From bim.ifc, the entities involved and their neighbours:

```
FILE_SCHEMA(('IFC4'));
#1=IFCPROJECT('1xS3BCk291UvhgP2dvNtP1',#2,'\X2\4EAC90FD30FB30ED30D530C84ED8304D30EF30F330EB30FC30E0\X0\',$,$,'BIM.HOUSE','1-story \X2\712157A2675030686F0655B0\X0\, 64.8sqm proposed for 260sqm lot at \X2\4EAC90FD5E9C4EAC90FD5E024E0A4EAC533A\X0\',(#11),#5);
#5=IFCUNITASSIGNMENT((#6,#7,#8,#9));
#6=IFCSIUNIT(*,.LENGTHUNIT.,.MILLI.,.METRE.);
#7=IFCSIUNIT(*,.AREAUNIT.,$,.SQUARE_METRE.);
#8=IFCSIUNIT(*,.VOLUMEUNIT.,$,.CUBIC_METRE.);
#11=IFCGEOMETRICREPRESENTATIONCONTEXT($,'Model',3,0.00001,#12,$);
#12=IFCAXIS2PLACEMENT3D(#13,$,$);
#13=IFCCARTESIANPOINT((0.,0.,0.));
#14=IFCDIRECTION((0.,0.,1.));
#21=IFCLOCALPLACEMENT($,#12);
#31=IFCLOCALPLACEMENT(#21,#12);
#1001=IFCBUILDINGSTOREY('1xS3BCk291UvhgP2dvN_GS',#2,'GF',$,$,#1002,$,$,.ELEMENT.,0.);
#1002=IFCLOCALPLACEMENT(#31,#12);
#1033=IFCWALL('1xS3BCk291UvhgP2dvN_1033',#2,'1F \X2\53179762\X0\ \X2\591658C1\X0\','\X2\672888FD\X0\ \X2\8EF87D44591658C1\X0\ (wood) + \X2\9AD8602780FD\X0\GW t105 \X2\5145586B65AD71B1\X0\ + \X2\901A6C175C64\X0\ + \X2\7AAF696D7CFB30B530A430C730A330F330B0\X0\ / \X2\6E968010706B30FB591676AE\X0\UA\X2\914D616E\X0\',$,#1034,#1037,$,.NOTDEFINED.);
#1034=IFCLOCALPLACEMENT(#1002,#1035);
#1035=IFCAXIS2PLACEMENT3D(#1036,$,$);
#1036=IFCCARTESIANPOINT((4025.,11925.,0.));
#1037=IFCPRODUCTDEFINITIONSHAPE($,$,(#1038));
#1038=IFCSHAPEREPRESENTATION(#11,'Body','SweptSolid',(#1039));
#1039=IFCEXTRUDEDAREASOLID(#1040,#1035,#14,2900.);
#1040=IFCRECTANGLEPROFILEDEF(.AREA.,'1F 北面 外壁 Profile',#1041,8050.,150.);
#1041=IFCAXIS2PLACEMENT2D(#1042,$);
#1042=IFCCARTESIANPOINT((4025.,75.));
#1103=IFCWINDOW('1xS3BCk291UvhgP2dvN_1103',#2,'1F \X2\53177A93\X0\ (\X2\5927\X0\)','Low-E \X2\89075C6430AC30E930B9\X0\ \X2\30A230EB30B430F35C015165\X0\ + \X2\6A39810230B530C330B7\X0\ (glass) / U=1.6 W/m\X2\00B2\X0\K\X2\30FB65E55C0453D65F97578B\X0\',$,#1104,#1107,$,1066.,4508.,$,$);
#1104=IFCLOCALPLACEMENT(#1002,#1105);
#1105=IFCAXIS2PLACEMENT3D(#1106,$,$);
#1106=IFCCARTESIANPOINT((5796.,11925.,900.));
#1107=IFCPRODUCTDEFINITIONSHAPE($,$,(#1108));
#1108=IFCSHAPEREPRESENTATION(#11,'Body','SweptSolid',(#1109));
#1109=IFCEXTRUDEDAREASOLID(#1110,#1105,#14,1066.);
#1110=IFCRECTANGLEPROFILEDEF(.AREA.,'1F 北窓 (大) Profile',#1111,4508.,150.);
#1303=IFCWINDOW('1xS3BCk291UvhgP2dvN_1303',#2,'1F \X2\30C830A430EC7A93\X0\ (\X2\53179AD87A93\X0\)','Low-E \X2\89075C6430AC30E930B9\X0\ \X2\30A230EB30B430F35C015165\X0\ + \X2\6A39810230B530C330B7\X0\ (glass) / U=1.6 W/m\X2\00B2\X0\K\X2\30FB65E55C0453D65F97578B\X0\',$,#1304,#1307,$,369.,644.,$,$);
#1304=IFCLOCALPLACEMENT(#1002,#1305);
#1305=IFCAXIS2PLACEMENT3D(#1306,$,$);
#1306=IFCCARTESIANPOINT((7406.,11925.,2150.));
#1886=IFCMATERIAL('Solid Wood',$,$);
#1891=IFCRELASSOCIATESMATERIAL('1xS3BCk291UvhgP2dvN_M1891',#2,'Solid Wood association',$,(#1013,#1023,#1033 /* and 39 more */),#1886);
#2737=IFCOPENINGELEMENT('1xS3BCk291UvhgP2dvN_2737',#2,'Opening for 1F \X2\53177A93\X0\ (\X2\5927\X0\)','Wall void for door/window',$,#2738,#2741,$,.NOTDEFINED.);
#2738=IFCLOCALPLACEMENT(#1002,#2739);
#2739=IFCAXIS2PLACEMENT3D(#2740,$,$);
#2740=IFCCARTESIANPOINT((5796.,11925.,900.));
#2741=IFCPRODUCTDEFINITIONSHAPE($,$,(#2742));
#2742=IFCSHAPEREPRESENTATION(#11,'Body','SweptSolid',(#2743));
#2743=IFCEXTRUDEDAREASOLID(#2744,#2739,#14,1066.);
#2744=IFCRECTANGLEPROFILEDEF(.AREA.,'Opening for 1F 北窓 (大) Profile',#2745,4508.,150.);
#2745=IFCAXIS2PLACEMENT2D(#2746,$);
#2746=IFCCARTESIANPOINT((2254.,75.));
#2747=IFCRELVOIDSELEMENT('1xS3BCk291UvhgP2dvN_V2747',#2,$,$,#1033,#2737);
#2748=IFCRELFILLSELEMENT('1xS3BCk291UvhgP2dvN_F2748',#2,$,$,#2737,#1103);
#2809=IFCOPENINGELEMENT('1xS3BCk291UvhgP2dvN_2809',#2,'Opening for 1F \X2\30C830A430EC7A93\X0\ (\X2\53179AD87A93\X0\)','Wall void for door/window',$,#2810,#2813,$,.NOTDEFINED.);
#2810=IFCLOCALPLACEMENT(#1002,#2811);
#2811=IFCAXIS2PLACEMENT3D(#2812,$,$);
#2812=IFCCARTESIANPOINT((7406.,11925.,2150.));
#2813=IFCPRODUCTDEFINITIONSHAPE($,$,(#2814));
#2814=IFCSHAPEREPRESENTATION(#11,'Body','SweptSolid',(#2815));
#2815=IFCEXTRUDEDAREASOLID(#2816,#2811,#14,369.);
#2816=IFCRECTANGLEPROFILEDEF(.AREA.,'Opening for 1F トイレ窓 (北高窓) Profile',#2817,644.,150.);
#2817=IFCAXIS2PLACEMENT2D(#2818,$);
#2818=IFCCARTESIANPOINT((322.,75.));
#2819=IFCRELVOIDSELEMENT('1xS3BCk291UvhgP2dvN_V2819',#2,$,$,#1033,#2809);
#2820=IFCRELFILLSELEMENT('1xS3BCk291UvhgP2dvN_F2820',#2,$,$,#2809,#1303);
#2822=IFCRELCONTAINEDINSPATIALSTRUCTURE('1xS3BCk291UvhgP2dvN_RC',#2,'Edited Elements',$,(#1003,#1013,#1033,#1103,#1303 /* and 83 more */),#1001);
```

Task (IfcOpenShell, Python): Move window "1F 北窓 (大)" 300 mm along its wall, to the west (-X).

```python
import ifcopenshell
import ifcopenshell.api.geometry
import ifcopenshell.util.placement
import ifcopenshell.util.unit

model = ifcopenshell.open("bim.ifc")
unit_scale = ifcopenshell.util.unit.calculate_unit_scale(model)

window = model.by_guid("1xS3BCk291UvhgP2dvN_1103")
opening = window.FillsVoids[0].RelatingOpeningElement
wall = opening.VoidsElements[0].RelatingBuildingElement

wall_matrix = ifcopenshell.util.placement.get_local_placement(wall.ObjectPlacement)
shift = wall_matrix[:3, 0] * -0.3 / unit_scale
before = ifcopenshell.util.placement.get_local_placement(window.ObjectPlacement)[:3, 3].copy()

# The window is not placed relative to its opening, so move both.
for product in (opening, window):
    matrix = ifcopenshell.util.placement.get_local_placement(product.ObjectPlacement)
    matrix[:3, 3] += shift
    ifcopenshell.api.geometry.edit_object_placement(model, product=product, matrix=matrix, is_si=False)

after = ifcopenshell.util.placement.get_local_placement(window.ObjectPlacement)[:3, 3]
print("window moved by", (after - before).round(3) + 0.0)

model.write("bim_rev.ifc")
```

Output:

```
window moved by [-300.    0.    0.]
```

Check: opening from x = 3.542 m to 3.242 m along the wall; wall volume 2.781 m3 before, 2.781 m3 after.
